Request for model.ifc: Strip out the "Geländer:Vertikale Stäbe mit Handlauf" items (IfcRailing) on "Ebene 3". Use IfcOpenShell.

First a look at what the model holds.

```python
import ifcopenshell
import ifcopenshell.util.element

model = ifcopenshell.open("model.ifc")
print(model.schema)
storey = next(s for s in model.by_type("IfcBuildingStorey") if s.Name == "Ebene 3")
railings = [e for e in ifcopenshell.util.element.get_decomposition(storey) if e.is_a("IfcRailing")]
seen = {}
for e in railings:
    element_type = ifcopenshell.util.element.get_type(e)
    name = element_type.Name if element_type not in (None, e) else None
    seen[name] = seen.get(name, 0) + 1
for name, count in sorted(seen.items(), key=str):
    print(count, "x", name)
```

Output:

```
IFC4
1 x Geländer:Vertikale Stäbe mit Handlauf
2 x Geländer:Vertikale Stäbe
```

```python
import ifcopenshell
import ifcopenshell.api.root
import ifcopenshell.util.element

model = ifcopenshell.open("model.ifc")

storey = next(s for s in model.by_type("IfcBuildingStorey") if s.Name == "Ebene 3")
railings = [e for e in ifcopenshell.util.element.get_decomposition(storey) if e.is_a("IfcRailing")]
targets = [e for e in railings if (t := ifcopenshell.util.element.get_type(e)) not in (None, e) and t.Name == "Geländer:Vertikale Stäbe mit Handlauf"]

for e in targets:
    ifcopenshell.api.root.remove_product(model, product=e)
print(len(targets), "removed")

model.write("model_updated.ifc")
```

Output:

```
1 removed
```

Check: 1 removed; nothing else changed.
